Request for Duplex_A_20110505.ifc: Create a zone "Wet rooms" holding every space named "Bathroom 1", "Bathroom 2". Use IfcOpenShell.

First a look at what the model holds.

```python
import ifcopenshell

model = ifcopenshell.open("Duplex_A_20110505.ifc")
print(model.schema)
seen = {}
for space in model.by_type("IfcSpace"):
    seen[space.LongName] = seen.get(space.LongName, 0) + 1
for name, count in sorted(seen.items(), key=str):
    print(count, "x", name)
print("zones:", [z.Name for z in model.by_type("IfcZone")][:20])
```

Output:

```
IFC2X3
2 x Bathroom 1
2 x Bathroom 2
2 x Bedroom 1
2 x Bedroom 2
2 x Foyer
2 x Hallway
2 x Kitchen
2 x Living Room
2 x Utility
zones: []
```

```python
import ifcopenshell
import ifcopenshell.api.group
import ifcopenshell.api.root

model = ifcopenshell.open("Duplex_A_20110505.ifc")

names = {"Bathroom 1", "Bathroom 2"}
spaces = [s for s in model.by_type("IfcSpace") if s.LongName in names]

zone = ifcopenshell.api.root.create_entity(model, ifc_class="IfcZone", name="Wet rooms")
ifcopenshell.api.group.assign_group(model, products=spaces, group=zone)
print(len(spaces), "spaces in", zone.Name)

model.write("Duplex_A_20110505_edited.ifc")
```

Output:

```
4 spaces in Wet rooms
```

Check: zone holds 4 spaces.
